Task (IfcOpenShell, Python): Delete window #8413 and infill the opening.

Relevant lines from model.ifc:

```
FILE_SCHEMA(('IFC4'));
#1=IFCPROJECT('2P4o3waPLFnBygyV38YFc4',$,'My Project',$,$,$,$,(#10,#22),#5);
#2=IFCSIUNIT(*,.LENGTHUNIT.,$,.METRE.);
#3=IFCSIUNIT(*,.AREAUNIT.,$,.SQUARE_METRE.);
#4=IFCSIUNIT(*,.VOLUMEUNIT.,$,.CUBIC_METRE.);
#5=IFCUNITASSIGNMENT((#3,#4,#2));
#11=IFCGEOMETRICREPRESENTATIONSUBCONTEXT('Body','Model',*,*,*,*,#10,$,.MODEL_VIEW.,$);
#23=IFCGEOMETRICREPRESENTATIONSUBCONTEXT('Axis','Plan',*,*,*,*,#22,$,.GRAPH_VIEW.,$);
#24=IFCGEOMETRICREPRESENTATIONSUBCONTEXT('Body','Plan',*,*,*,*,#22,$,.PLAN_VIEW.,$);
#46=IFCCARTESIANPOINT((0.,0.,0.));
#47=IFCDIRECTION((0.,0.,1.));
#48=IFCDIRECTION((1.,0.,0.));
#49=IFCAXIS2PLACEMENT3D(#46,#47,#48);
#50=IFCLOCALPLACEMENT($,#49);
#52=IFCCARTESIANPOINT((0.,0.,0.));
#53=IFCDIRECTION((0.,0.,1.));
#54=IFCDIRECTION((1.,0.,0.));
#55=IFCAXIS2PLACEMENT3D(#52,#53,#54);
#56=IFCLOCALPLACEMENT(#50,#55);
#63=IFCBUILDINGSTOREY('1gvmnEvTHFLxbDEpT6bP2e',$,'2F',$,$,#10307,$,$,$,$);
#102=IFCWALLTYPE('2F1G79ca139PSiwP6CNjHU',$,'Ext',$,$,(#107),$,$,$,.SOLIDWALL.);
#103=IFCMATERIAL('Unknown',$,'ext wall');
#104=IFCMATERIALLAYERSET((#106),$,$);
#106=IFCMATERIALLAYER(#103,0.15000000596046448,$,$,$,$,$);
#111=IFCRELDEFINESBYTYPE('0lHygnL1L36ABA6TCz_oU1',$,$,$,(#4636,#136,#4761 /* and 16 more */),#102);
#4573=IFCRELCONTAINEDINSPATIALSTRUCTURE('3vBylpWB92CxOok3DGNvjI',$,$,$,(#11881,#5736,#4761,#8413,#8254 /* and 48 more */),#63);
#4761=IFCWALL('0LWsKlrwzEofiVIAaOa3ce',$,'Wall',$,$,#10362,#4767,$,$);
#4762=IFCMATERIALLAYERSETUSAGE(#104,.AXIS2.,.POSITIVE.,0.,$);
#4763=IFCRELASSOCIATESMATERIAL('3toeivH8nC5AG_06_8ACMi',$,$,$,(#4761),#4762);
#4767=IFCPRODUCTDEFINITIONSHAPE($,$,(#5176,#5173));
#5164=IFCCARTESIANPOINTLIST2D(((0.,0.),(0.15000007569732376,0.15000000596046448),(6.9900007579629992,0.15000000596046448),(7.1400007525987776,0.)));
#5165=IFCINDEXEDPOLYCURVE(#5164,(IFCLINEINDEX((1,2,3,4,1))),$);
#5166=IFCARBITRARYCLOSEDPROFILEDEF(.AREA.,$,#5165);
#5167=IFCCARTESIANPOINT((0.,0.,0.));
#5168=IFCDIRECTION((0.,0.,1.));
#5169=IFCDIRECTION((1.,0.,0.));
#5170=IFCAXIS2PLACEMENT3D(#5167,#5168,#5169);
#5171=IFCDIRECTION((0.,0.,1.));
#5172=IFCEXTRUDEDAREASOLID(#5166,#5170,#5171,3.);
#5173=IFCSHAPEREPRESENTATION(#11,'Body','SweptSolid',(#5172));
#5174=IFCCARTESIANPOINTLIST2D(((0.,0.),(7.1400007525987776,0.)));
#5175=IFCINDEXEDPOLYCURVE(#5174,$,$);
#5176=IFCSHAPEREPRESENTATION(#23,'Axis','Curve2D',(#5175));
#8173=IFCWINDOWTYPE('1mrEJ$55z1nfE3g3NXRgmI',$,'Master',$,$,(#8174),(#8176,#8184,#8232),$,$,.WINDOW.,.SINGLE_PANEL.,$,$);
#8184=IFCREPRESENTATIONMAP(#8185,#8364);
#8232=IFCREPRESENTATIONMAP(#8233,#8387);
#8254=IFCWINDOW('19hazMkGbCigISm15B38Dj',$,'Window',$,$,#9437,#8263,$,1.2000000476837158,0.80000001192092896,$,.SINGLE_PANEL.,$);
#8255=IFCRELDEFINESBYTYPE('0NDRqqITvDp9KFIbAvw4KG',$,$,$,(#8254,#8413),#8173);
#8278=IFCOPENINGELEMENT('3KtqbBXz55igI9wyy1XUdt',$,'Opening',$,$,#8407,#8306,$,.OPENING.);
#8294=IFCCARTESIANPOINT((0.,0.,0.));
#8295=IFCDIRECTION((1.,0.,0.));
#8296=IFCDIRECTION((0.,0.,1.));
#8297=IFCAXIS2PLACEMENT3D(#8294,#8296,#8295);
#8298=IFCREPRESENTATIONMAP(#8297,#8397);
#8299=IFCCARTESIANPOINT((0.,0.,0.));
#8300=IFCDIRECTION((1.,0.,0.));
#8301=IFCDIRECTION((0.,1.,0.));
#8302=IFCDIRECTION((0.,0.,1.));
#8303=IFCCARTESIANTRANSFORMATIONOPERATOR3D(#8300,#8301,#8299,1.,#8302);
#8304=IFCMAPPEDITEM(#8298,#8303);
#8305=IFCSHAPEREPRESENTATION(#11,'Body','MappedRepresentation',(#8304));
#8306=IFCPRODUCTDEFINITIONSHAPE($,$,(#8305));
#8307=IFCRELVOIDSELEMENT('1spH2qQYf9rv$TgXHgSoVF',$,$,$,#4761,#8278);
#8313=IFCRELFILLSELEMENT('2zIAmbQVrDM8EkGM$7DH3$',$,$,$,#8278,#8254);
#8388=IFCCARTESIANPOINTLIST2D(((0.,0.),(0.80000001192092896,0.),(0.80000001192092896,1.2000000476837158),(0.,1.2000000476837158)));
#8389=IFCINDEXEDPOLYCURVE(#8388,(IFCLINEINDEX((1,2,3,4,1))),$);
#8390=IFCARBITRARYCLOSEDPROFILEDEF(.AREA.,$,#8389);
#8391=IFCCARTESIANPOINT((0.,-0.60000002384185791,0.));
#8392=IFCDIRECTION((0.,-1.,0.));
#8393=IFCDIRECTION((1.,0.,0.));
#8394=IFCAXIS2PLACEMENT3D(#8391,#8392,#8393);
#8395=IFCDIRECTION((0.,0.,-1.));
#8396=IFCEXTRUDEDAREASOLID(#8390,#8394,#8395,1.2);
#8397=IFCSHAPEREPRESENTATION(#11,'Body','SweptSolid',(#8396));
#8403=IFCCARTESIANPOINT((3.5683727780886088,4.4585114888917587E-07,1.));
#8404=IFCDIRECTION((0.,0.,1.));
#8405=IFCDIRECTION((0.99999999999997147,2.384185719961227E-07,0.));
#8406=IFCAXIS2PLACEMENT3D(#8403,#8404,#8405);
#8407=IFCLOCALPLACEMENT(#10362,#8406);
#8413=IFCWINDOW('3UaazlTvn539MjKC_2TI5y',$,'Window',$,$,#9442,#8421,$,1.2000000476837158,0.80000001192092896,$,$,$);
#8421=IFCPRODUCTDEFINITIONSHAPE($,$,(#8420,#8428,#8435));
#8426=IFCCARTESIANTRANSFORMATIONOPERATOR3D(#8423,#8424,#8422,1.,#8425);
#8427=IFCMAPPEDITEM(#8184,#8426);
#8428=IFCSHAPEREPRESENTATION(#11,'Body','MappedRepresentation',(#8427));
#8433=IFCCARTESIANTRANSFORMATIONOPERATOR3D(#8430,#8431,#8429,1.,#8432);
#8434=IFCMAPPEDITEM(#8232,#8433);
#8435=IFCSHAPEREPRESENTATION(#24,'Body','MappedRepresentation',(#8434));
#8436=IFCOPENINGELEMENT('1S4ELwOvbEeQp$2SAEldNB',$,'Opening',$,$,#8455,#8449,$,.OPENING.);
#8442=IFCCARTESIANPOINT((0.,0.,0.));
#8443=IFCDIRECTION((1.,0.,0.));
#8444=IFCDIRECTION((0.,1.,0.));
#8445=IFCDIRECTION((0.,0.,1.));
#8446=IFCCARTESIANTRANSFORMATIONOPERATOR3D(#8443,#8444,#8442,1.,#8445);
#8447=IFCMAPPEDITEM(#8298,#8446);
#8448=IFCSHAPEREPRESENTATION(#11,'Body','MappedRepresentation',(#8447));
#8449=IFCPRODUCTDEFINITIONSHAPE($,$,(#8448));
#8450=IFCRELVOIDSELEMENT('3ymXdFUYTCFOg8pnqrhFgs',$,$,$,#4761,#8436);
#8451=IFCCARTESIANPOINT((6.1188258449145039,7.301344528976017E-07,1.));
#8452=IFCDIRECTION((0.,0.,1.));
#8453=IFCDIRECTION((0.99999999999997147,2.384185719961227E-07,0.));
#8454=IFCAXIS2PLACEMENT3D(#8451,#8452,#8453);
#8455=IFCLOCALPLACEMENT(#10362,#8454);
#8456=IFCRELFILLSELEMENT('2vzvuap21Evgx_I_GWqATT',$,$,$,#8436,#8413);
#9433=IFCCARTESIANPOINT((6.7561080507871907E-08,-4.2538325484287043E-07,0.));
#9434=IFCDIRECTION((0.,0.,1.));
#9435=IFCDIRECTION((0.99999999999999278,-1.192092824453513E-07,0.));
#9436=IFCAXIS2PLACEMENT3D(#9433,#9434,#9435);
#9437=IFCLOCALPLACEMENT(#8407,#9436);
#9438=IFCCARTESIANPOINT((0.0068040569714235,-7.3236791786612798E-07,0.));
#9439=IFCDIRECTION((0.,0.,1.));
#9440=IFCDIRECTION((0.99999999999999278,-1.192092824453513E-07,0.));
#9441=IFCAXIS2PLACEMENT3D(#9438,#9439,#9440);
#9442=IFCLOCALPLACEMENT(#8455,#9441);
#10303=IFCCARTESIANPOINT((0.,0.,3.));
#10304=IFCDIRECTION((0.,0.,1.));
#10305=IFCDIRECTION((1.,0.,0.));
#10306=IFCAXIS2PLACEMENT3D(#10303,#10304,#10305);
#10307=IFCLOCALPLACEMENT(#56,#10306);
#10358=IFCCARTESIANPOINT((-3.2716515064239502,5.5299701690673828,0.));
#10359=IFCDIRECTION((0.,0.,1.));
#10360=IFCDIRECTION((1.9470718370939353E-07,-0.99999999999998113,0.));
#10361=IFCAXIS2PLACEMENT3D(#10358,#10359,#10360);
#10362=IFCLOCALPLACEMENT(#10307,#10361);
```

```python
import ifcopenshell
import ifcopenshell.api.feature
import ifcopenshell.api.root
import ifcopenshell.geom
import ifcopenshell.util.shape

model = ifcopenshell.open("model.ifc")
settings = ifcopenshell.geom.settings()


def volume(element):
    """Net volume in cubic metres, openings subtracted."""
    shape = ifcopenshell.geom.create_shape(settings, element)
    return ifcopenshell.util.shape.get_volume(shape.geometry)


window = model.by_guid("3UaazlTvn539MjKC_2TI5y")
opening = window.FillsVoids[0].RelatingOpeningElement
wall = opening.VoidsElements[0].RelatingBuildingElement
before = volume(wall)

ifcopenshell.api.root.remove_product(model, product=window)
ifcopenshell.api.feature.remove_feature(model, feature=opening)

after = volume(wall)

print(f"wall volume {before:.3f} -> {after:.3f} m3")

model.write("model-out.ifc")
```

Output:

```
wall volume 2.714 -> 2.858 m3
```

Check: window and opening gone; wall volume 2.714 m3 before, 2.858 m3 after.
